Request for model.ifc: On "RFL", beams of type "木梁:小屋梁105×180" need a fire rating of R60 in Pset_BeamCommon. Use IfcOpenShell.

First a look at what the model holds.

```python
import ifcopenshell
import ifcopenshell.util.element

model = ifcopenshell.open("model.ifc")
print(model.schema)
storey = next(s for s in model.by_type("IfcBuildingStorey") if s.Name == "RFL")
beams = [e for e in ifcopenshell.util.element.get_decomposition(storey) if e.is_a("IfcBeam")]
seen = {}
for e in beams:
    element_type = ifcopenshell.util.element.get_type(e)
    key = (element_type.Name if element_type != e and element_type else None, ifcopenshell.util.element.get_pset(e, "Pset_BeamCommon", "FireRating"))
    seen[key] = seen.get(key, 0) + 1
for (name, value), count in sorted(seen.items(), key=str):
    print(count, "x", name, "|", value)
```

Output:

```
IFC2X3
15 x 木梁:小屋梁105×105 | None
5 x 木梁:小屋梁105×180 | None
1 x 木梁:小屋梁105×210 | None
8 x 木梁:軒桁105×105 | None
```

```python
import ifcopenshell
import ifcopenshell.api.pset
import ifcopenshell.util.element

model = ifcopenshell.open("model.ifc")

storey = next(s for s in model.by_type("IfcBuildingStorey") if s.Name == "RFL")
beams = [e for e in ifcopenshell.util.element.get_decomposition(storey) if e.is_a("IfcBeam")]

count = 0
for e in beams:
    element_type = ifcopenshell.util.element.get_type(e)
    if element_type in (None, e) or element_type.Name != "木梁:小屋梁105×180":
        continue
    # add_pset returns the element's existing set when there is one.
    pset = ifcopenshell.api.pset.add_pset(model, product=e, name="Pset_BeamCommon")
    ifcopenshell.api.pset.edit_pset(model, pset=pset, properties={"FireRating": "R60"})
    count += 1

print(count, "beams updated")

model.write("model-out.ifc")
```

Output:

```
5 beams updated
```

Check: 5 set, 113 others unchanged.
